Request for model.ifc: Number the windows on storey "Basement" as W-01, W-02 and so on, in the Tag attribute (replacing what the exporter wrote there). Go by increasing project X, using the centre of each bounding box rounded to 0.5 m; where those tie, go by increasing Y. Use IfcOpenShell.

First a look at what the model holds.

```python
import ifcopenshell
import ifcopenshell.util.element
import ifcopenshell.util.placement

model = ifcopenshell.open("model.ifc")
print(model.schema)
storey = next(s for s in model.by_type("IfcBuildingStorey") if s.Name == "Basement")
windows = [e for e in ifcopenshell.util.element.get_decomposition(storey) if e.is_a("IfcWindow")]
for e in sorted(windows, key=lambda e: e.id()):
    origin = ifcopenshell.util.placement.get_local_placement(e.ObjectPlacement)[:3, 3]
    print(e.id(), e.Tag, e.Name, origin.round(2) + 0.0, sep=" | ")
```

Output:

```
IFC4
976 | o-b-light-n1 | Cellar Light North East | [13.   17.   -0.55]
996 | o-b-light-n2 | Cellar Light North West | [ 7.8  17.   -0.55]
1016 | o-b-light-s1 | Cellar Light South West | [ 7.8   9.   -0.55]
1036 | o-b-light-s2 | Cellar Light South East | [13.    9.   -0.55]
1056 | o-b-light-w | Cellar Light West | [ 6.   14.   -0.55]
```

```python
import ifcopenshell
import ifcopenshell.geom
import ifcopenshell.util.element
import ifcopenshell.util.shape

model = ifcopenshell.open("model.ifc")
settings = ifcopenshell.geom.settings()
settings.set("use-world-coords", True)


def centre(element):
    shape = ifcopenshell.geom.create_shape(settings, element)
    return ifcopenshell.util.shape.get_bbox_centroid(shape.geometry)


storey = next(s for s in model.by_type("IfcBuildingStorey") if s.Name == "Basement")
windows = [e for e in ifcopenshell.util.element.get_decomposition(storey) if e.is_a("IfcWindow")]

# Insertion points can sit at a corner or the storey origin, so sort by the geometry (in metres).
centres = {e: centre(e) for e in windows}
windows.sort(key=lambda e: (round(centres[e][0] / 0.5), centres[e][1]))

for i, e in enumerate(windows, start=1):
    number = f"W-{i:02d}"
    e.Tag = number
    print(e.id(), number)

model.write("model_updated.ifc")
```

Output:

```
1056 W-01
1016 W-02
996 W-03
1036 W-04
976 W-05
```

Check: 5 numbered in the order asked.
